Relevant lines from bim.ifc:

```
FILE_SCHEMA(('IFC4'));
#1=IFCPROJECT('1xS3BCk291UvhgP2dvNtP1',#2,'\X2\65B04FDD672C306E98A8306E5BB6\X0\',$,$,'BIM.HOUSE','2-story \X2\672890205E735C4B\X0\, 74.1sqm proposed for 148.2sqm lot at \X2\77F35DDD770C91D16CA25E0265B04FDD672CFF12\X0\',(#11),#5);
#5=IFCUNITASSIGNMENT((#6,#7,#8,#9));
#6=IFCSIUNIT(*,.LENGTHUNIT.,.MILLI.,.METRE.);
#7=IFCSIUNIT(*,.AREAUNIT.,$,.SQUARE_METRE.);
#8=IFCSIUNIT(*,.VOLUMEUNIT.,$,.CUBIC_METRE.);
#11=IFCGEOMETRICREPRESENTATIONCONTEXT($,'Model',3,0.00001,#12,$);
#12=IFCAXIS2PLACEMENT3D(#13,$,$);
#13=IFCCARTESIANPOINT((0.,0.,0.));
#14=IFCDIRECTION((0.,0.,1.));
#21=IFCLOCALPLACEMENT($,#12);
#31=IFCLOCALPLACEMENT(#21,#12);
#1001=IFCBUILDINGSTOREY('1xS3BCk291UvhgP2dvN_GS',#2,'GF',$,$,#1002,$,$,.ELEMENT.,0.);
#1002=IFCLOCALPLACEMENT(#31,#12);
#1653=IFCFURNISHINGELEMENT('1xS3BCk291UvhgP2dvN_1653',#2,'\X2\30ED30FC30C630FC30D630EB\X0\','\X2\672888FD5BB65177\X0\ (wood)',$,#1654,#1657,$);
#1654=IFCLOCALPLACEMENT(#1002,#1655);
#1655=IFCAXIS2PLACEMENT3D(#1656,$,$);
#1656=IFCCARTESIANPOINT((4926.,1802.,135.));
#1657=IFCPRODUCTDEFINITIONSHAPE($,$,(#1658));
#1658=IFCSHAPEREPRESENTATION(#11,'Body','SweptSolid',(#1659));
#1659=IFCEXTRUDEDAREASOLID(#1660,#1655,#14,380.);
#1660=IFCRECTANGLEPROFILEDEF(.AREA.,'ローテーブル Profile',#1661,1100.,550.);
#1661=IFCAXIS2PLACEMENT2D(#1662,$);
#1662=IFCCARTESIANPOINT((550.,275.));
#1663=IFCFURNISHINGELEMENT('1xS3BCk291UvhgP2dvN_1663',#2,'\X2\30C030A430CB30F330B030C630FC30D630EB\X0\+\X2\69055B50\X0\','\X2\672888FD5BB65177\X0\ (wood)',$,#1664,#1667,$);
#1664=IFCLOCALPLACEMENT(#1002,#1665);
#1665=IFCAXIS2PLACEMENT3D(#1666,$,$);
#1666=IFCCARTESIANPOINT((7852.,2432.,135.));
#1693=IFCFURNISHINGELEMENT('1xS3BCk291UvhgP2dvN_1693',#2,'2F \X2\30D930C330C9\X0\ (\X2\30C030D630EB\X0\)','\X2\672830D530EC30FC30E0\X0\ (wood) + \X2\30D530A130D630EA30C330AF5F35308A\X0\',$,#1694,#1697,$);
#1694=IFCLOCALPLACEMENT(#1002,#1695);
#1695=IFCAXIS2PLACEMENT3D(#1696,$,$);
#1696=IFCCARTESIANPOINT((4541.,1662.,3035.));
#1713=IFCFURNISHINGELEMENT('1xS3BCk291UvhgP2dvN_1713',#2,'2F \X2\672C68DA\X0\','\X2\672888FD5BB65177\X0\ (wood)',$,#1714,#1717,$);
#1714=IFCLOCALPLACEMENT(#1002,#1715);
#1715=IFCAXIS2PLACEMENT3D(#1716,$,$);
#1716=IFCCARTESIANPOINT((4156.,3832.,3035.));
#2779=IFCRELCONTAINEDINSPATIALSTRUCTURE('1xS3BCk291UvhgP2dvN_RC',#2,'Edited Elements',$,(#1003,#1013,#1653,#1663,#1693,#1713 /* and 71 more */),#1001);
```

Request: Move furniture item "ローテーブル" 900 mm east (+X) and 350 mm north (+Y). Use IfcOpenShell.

```python
import ifcopenshell
import ifcopenshell.api.geometry
import ifcopenshell.util.placement
import ifcopenshell.util.unit

model = ifcopenshell.open("bim.ifc")
unit_scale = ifcopenshell.util.unit.calculate_unit_scale(model)

item = model.by_id(1653)
matrix = ifcopenshell.util.placement.get_local_placement(item.ObjectPlacement)
matrix[0, 3] += 0.9 / unit_scale
matrix[1, 3] += 0.35 / unit_scale
ifcopenshell.api.geometry.edit_object_placement(model, product=item, matrix=matrix, is_si=False)

print(ifcopenshell.util.placement.get_local_placement(item.ObjectPlacement).round(3) + 0.0)

model.write("bim_v2.ifc")
```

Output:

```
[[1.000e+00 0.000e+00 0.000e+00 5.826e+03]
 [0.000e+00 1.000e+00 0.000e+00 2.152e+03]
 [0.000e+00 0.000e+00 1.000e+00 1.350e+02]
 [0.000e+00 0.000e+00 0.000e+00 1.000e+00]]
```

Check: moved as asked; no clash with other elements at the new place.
